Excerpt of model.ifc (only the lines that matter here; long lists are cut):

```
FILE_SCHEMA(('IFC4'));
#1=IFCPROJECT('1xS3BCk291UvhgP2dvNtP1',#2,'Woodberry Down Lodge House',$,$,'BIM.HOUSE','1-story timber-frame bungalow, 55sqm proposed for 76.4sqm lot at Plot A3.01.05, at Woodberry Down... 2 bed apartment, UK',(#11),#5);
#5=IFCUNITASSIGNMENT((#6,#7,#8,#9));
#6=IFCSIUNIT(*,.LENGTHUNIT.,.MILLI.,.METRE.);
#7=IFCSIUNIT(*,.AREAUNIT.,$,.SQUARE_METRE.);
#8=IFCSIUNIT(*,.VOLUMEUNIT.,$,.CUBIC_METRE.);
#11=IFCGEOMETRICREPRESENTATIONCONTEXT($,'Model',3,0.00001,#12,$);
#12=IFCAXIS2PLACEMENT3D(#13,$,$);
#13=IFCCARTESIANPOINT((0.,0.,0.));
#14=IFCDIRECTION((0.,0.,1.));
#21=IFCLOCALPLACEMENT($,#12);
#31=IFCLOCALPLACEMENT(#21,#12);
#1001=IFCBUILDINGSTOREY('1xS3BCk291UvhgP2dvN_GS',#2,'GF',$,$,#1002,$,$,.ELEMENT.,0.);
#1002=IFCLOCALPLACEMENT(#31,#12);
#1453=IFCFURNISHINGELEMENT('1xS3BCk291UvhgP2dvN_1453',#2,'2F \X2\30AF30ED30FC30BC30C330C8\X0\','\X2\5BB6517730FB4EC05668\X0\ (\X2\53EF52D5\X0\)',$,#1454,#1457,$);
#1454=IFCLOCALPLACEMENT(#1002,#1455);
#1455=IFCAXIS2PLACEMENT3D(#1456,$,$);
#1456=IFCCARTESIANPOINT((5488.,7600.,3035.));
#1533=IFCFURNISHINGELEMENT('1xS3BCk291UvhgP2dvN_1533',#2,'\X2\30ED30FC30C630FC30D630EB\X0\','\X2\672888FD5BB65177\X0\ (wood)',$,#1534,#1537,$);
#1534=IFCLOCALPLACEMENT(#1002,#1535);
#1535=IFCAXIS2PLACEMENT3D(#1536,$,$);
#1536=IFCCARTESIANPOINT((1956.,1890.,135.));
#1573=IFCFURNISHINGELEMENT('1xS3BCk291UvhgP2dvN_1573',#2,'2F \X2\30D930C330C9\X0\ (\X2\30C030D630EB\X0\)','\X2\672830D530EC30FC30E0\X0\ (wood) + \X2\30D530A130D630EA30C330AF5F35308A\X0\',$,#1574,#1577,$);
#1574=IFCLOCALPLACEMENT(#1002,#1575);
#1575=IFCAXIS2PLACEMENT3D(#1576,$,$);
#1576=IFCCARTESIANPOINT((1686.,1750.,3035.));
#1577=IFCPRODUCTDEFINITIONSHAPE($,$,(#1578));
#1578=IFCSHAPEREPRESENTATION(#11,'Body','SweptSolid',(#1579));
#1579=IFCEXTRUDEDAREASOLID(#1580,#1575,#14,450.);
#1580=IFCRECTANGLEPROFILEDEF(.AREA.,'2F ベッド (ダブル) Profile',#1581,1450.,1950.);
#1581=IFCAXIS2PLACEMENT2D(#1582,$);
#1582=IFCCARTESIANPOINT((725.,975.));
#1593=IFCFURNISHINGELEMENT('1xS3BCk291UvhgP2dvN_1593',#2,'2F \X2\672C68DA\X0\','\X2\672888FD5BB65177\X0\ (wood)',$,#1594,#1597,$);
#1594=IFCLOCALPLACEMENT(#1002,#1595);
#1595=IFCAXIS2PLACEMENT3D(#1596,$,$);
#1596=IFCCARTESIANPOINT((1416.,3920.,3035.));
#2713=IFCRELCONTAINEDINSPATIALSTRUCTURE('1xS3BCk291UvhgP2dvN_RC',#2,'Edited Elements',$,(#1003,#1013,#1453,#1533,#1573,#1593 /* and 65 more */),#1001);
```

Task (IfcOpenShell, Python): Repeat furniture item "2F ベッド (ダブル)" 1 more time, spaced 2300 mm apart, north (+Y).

```python
import numpy as np
import ifcopenshell
import ifcopenshell.api.geometry
import ifcopenshell.api.root
import ifcopenshell.util.element
import ifcopenshell.util.placement

model = ifcopenshell.open("model.ifc")


def reuse_history(source, copy):
    """copy_class also copies each property set's owner history, people and application; keep the originals."""
    for rel in copy.IsDefinedBy:
        if rel.is_a("IfcRelDefinesByProperties") and (history := rel.RelatingPropertyDefinition.OwnerHistory):
            rel.RelatingPropertyDefinition.OwnerHistory = source.OwnerHistory
            ifcopenshell.util.element.remove_deep2(model, history)


source = model.by_guid("1xS3BCk291UvhgP2dvN_1573")
base = ifcopenshell.util.placement.get_local_placement(source.ObjectPlacement)
step = np.array([0.0, 1.0, 0.0]) * 2300.0

for i in range(1, 2):
    copy = ifcopenshell.api.root.copy_class(model, product=source)
    copy.Representation = ifcopenshell.util.element.copy_deep(
        model, source.Representation, exclude=["IfcGeometricRepresentationContext", "IfcRepresentationMap"]
    )
    reuse_history(source, copy)
    matrix = base.copy()
    matrix[:3, 3] += i * step
    print("added at", matrix[:3, 3].round(3) + 0.0)
    ifcopenshell.api.geometry.edit_object_placement(model, product=copy, matrix=matrix, is_si=False)

model.write("model_rev.ifc")
```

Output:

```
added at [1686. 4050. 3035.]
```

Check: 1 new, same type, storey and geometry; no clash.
